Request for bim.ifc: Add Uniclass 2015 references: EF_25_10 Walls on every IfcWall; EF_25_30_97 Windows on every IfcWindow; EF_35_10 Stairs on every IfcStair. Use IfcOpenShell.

First a look at what the model holds.

```python
import ifcopenshell

model = ifcopenshell.open("bim.ifc")
print(model.schema)
print("classifications:", [c.Name for c in model.by_type("IfcClassification")])
for ifc_class in ("IfcDoor", "IfcRoof", "IfcStair", "IfcWall", "IfcWindow"):
    print(ifc_class, len(model.by_type(ifc_class)))
```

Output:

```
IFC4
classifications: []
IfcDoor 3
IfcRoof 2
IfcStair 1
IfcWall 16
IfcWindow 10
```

```python
import ifcopenshell
import ifcopenshell.api.classification

model = ifcopenshell.open("bim.ifc")

system = ifcopenshell.api.classification.add_classification(model, classification="Uniclass 2015")

codes = {
    "IfcWall": ("EF_25_10", "Walls"),
    "IfcWindow": ("EF_25_30_97", "Windows"),
    "IfcStair": ("EF_35_10", "Stairs"),
}
for ifc_class, (code, name) in codes.items():
    products = model.by_type(ifc_class)
    ifcopenshell.api.classification.add_reference(
        model, products=products, classification=system, identification=code, name=name
    )
    print(code, len(products))

model.write("bim-out.ifc")
```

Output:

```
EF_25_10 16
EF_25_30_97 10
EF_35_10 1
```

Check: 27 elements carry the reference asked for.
